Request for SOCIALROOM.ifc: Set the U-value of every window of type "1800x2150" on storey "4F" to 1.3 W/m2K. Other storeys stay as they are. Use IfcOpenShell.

First a look at what the model holds.

```python
import ifcopenshell
import ifcopenshell.util.element

model = ifcopenshell.open("SOCIALROOM.ifc")
print(model.schema)
storey = next(s for s in model.by_type("IfcBuildingStorey") if s.Name == "4F")
windows = [e for e in ifcopenshell.util.element.get_decomposition(storey) if e.is_a("IfcWindow")]
seen = {}
for e in windows:
    element_type = ifcopenshell.util.element.get_type(e)
    key = (element_type.Name if element_type != e and element_type else None, ifcopenshell.util.element.get_pset(e, "Pset_WindowCommon", "ThermalTransmittance"))
    seen[key] = seen.get(key, 0) + 1
for (name, value), count in sorted(seen.items(), key=str):
    print(count, "x", name, "|", value)
```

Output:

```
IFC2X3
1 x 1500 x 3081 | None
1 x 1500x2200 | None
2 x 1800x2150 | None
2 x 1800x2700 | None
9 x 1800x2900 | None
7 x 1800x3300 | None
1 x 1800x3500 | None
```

```python
import ifcopenshell
import ifcopenshell.api.pset
import ifcopenshell.util.element

model = ifcopenshell.open("SOCIALROOM.ifc")

storey = next(s for s in model.by_type("IfcBuildingStorey") if s.Name == "4F")
windows = [e for e in ifcopenshell.util.element.get_decomposition(storey) if e.is_a("IfcWindow")]

count = 0
for e in windows:
    element_type = ifcopenshell.util.element.get_type(e)
    if element_type in (None, e) or element_type.Name != "1800x2150":
        continue
    # add_pset returns the element's existing set when there is one.
    pset = ifcopenshell.api.pset.add_pset(model, product=e, name="Pset_WindowCommon")
    ifcopenshell.api.pset.edit_pset(model, pset=pset, properties={"ThermalTransmittance": 1.3})
    count += 1

print(count, "windows updated")

model.write("SOCIALROOM-out.ifc")
```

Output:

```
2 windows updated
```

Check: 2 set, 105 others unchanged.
